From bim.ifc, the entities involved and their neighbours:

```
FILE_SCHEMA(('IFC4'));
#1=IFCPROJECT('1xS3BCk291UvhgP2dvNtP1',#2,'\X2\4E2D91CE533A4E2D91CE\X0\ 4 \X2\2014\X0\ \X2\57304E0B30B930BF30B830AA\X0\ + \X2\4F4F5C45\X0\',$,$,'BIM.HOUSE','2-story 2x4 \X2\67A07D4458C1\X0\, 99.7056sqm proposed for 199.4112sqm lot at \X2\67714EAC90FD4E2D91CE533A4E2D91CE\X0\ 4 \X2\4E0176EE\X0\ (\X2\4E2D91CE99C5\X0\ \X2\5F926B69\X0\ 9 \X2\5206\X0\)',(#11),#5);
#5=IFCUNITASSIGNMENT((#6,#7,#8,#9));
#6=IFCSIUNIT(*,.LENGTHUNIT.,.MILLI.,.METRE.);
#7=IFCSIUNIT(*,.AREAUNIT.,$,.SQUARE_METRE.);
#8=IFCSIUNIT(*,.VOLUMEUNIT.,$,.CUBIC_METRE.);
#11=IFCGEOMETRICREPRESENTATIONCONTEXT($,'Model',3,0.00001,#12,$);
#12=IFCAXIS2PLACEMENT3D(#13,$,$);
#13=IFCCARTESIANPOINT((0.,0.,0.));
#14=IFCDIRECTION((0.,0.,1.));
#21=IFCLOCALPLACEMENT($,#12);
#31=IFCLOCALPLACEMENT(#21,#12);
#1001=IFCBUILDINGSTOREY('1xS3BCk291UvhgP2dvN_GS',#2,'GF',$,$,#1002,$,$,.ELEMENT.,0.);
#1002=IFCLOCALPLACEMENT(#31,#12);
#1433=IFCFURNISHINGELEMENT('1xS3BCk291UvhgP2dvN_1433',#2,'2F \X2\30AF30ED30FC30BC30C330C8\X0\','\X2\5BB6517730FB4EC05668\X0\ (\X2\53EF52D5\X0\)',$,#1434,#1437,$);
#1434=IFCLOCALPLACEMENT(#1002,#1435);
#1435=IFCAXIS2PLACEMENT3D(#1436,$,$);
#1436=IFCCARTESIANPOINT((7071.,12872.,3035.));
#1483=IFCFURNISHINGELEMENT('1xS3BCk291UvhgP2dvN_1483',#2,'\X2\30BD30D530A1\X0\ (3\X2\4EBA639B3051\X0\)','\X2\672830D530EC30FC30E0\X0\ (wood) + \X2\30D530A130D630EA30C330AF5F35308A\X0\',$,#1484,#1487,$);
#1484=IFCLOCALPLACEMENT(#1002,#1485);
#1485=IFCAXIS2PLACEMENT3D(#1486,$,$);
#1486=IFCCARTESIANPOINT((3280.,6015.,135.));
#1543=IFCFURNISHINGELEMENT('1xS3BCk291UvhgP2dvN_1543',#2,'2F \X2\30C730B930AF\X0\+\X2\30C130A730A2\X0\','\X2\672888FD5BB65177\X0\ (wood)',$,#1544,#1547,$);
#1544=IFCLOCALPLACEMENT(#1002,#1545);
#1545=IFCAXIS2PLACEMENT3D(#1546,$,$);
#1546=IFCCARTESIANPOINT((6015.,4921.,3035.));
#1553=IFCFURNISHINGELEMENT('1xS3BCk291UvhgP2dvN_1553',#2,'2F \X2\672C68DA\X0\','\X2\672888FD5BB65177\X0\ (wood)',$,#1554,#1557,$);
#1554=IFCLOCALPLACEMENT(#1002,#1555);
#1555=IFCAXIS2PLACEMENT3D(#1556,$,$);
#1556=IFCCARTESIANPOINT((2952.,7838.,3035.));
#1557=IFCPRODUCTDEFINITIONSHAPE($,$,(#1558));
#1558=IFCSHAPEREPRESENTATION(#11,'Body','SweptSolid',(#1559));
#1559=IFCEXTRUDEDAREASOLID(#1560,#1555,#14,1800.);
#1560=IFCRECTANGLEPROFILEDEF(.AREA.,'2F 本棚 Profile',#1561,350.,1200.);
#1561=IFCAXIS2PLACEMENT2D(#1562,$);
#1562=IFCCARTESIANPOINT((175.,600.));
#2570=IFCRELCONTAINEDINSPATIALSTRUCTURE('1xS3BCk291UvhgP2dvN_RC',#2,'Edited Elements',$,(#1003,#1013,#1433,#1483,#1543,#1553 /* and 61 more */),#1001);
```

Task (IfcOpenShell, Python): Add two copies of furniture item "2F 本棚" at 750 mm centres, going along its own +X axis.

```python
import ifcopenshell
import ifcopenshell.api.geometry
import ifcopenshell.api.root
import ifcopenshell.util.element
import ifcopenshell.util.placement
import ifcopenshell.util.unit

model = ifcopenshell.open("bim.ifc")
unit_scale = ifcopenshell.util.unit.calculate_unit_scale(model)


def reuse_history(source, copy):
    """copy_class also copies each property set's owner history, people and application; keep the originals."""
    for rel in copy.IsDefinedBy:
        if rel.is_a("IfcRelDefinesByProperties") and (history := rel.RelatingPropertyDefinition.OwnerHistory):
            rel.RelatingPropertyDefinition.OwnerHistory = source.OwnerHistory
            ifcopenshell.util.element.remove_deep2(model, history)


source = model.by_id(1553)
base = ifcopenshell.util.placement.get_local_placement(source.ObjectPlacement)
step = base[:3, 0] * 0.75 / unit_scale

for i in range(1, 3):
    copy = ifcopenshell.api.root.copy_class(model, product=source)
    copy.Representation = ifcopenshell.util.element.copy_deep(
        model, source.Representation, exclude=["IfcGeometricRepresentationContext", "IfcRepresentationMap"]
    )
    reuse_history(source, copy)
    matrix = base.copy()
    matrix[:3, 3] += i * step
    print("added at", matrix[:3, 3].round(3) + 0.0)
    ifcopenshell.api.geometry.edit_object_placement(model, product=copy, matrix=matrix, is_si=False)

model.write("bim_updated.ifc")
```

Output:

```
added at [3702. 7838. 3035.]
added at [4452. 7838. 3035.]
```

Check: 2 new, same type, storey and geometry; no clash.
